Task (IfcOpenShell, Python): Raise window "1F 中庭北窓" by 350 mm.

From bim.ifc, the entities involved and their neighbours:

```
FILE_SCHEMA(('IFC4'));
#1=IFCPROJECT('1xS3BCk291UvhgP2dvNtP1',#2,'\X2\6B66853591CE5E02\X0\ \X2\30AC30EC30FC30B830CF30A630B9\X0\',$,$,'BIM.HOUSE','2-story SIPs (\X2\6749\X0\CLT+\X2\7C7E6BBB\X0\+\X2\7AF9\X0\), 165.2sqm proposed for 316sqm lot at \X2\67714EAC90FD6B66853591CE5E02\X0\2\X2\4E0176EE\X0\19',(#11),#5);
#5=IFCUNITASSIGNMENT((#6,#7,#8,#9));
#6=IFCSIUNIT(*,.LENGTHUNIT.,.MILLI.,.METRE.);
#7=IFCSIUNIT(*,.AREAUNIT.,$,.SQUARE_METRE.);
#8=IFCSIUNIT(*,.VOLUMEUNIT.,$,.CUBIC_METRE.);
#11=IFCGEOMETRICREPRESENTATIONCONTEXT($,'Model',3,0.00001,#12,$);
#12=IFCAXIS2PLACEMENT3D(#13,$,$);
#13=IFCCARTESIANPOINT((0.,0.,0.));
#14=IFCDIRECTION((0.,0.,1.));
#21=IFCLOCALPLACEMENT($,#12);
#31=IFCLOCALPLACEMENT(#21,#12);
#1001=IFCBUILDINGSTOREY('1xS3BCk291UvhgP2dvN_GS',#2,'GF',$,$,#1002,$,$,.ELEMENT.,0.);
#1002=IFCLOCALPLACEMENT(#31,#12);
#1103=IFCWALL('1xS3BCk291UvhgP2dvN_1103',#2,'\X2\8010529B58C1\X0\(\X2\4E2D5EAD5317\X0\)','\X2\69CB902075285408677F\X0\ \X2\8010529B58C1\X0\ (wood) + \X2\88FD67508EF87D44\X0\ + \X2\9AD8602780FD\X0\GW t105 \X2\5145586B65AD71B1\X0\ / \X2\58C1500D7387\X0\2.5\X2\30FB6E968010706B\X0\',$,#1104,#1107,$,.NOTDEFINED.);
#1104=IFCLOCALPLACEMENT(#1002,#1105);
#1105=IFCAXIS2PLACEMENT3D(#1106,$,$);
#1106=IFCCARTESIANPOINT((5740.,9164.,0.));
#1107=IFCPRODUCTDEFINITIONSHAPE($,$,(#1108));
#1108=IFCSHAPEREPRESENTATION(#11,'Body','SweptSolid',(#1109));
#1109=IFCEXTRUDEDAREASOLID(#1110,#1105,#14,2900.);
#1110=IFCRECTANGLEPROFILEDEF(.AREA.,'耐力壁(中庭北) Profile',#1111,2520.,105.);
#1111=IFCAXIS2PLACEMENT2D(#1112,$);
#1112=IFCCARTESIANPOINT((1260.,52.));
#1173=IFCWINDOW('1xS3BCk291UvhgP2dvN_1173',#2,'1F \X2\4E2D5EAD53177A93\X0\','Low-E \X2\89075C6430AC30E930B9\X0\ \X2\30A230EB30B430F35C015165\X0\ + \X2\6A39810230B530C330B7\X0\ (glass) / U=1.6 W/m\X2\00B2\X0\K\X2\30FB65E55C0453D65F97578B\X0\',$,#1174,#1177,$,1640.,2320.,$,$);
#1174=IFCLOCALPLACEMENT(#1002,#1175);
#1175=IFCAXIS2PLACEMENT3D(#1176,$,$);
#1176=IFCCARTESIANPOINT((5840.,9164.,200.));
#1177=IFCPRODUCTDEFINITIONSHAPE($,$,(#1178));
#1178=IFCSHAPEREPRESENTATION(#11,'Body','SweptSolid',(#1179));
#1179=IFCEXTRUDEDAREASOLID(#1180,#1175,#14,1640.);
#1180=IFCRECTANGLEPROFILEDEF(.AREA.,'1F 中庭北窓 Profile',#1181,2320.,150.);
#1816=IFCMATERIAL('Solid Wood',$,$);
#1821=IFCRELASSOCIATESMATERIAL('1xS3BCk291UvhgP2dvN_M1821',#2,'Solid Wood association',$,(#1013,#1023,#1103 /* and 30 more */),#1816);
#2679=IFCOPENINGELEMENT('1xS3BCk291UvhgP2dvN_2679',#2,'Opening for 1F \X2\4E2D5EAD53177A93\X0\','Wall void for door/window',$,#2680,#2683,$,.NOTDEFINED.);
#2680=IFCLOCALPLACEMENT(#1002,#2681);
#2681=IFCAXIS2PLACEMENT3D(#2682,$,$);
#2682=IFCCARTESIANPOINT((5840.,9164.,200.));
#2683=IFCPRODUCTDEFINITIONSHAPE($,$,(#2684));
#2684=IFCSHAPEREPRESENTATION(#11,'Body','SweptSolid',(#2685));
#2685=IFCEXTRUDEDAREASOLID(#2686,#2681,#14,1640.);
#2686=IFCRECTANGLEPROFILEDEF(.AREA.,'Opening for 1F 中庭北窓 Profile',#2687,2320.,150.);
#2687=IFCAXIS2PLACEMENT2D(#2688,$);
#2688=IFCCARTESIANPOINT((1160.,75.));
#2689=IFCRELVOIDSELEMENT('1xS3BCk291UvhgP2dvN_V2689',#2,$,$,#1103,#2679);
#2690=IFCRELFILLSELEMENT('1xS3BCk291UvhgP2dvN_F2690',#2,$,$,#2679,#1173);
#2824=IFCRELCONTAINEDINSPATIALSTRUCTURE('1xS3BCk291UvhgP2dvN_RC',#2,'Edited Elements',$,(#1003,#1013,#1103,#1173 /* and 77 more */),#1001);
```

```python
import numpy as np
import ifcopenshell
import ifcopenshell.api.geometry
import ifcopenshell.util.placement
import ifcopenshell.util.unit

model = ifcopenshell.open("bim.ifc")
unit_scale = ifcopenshell.util.unit.calculate_unit_scale(model)

window = model.by_id(1173)
opening = window.FillsVoids[0].RelatingOpeningElement
dz = 0.35 / unit_scale

shift = np.array([0.0, 0.0, dz])
# The window is not placed relative to its opening, so move both.
for product in (opening, window):
    matrix = ifcopenshell.util.placement.get_local_placement(product.ObjectPlacement)
    matrix[:3, 3] += shift
    ifcopenshell.api.geometry.edit_object_placement(model, product=product, matrix=matrix, is_si=False)

print(f"moved by {dz * unit_scale:+.3f} m")

model.write("bim-out.ifc")
```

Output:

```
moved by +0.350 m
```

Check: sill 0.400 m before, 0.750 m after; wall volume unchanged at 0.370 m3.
